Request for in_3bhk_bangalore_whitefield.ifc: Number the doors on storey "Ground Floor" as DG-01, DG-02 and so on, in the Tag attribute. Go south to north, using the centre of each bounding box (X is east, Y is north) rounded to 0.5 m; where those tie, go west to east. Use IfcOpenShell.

First a look at what the model holds.

```python
import ifcopenshell
import ifcopenshell.util.element
import ifcopenshell.util.placement

model = ifcopenshell.open("in_3bhk_bangalore_whitefield.ifc")
print(model.schema)
storey = next(s for s in model.by_type("IfcBuildingStorey") if s.Name == "Ground Floor")
doors = [e for e in ifcopenshell.util.element.get_decomposition(storey) if e.is_a("IfcDoor")]
for e in sorted(doors, key=lambda e: e.id()):
    origin = ifcopenshell.util.placement.get_local_placement(e.ObjectPlacement)[:3, 3]
    print(e.id(), e.Tag, e.Name, origin.round(2) + 0.0, sep=" | ")
```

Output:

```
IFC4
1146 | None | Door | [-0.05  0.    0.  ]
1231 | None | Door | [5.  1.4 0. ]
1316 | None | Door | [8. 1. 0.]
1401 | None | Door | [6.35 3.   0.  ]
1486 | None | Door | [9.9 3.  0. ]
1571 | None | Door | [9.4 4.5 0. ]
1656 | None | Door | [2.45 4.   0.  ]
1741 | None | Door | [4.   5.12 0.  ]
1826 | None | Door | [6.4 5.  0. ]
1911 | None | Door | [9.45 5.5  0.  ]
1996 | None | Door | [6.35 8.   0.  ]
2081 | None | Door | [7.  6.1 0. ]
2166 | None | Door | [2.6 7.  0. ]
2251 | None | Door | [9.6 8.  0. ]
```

```python
import ifcopenshell
import ifcopenshell.geom
import ifcopenshell.util.element
import ifcopenshell.util.shape

model = ifcopenshell.open("in_3bhk_bangalore_whitefield.ifc")
settings = ifcopenshell.geom.settings()
settings.set("use-world-coords", True)


def centre(element):
    shape = ifcopenshell.geom.create_shape(settings, element)
    return ifcopenshell.util.shape.get_bbox_centroid(shape.geometry)


storey = next(s for s in model.by_type("IfcBuildingStorey") if s.Name == "Ground Floor")
doors = [e for e in ifcopenshell.util.element.get_decomposition(storey) if e.is_a("IfcDoor")]

# Insertion points can sit at a corner or the storey origin, so sort by the geometry (in metres).
centres = {e: centre(e) for e in doors}
doors.sort(key=lambda e: (round(centres[e][1] / 0.5), centres[e][0]))

for i, e in enumerate(doors, start=1):
    number = f"DG-{i:02d}"
    e.Tag = number
    print(e.id(), number)

model.write("in_3bhk_bangalore_whitefield_edited.ifc")
```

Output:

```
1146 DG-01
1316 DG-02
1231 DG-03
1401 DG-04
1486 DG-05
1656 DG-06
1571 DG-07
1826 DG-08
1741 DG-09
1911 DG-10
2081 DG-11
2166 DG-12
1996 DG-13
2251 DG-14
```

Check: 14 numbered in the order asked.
